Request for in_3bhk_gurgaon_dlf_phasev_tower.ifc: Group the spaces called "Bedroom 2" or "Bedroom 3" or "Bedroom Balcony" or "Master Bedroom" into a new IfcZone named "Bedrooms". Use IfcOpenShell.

First a look at what the model holds.

```python
import ifcopenshell

model = ifcopenshell.open("in_3bhk_gurgaon_dlf_phasev_tower.ifc")
print(model.schema)
seen = {}
for space in model.by_type("IfcSpace"):
    seen[space.LongName] = seen.get(space.LongName, 0) + 1
for name, count in sorted(seen.items(), key=str):
    print(count, "x", name)
print("zones:", [z.Name for z in model.by_type("IfcZone")][:20])
```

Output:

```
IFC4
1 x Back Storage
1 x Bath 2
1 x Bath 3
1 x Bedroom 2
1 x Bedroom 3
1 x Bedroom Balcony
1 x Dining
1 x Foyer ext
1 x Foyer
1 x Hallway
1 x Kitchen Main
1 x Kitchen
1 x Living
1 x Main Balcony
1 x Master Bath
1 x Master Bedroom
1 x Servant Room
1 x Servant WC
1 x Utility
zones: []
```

```python
import ifcopenshell
import ifcopenshell.api.group
import ifcopenshell.api.root

model = ifcopenshell.open("in_3bhk_gurgaon_dlf_phasev_tower.ifc")

names = {"Bedroom 2", "Bedroom 3", "Bedroom Balcony", "Master Bedroom"}
spaces = [s for s in model.by_type("IfcSpace") if s.LongName in names]

zone = ifcopenshell.api.root.create_entity(model, ifc_class="IfcZone", name="Bedrooms")
ifcopenshell.api.group.assign_group(model, products=spaces, group=zone)
print(len(spaces), "spaces in", zone.Name)

model.write("in_3bhk_gurgaon_dlf_phasev_tower_rev.ifc")
```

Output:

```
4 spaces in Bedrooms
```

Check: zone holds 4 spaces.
